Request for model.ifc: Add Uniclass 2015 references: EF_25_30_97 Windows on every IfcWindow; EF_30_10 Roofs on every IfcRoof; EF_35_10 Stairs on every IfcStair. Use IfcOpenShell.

First a look at what the model holds.

```python
import ifcopenshell

model = ifcopenshell.open("model.ifc")
print(model.schema)
print("classifications:", [c.Name for c in model.by_type("IfcClassification")])
for ifc_class in ("IfcDoor", "IfcRoof", "IfcStair", "IfcWall", "IfcWindow"):
    print(ifc_class, len(model.by_type(ifc_class)))
```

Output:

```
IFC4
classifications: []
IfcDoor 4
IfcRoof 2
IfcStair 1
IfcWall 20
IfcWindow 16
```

```python
import ifcopenshell
import ifcopenshell.api.classification

model = ifcopenshell.open("model.ifc")

system = ifcopenshell.api.classification.add_classification(model, classification="Uniclass 2015")

codes = {
    "IfcWindow": ("EF_25_30_97", "Windows"),
    "IfcRoof": ("EF_30_10", "Roofs"),
    "IfcStair": ("EF_35_10", "Stairs"),
}
for ifc_class, (code, name) in codes.items():
    products = model.by_type(ifc_class)
    ifcopenshell.api.classification.add_reference(
        model, products=products, classification=system, identification=code, name=name
    )
    print(code, len(products))

model.write("model-out.ifc")
```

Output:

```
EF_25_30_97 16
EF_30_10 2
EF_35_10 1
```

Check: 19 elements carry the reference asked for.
